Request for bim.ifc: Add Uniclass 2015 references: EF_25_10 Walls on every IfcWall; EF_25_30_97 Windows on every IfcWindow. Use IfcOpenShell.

First a look at what the model holds.

```python
import ifcopenshell

model = ifcopenshell.open("bim.ifc")
print(model.schema)
print("classifications:", [c.Name for c in model.by_type("IfcClassification")])
for ifc_class in ("IfcDoor", "IfcRoof", "IfcStair", "IfcWall", "IfcWindow"):
    print(ifc_class, len(model.by_type(ifc_class)))
```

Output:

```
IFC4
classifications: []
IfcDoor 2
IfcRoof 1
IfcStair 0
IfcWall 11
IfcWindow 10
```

```python
import ifcopenshell
import ifcopenshell.api.classification

model = ifcopenshell.open("bim.ifc")

system = ifcopenshell.api.classification.add_classification(model, classification="Uniclass 2015")

codes = {
    "IfcWall": ("EF_25_10", "Walls"),
    "IfcWindow": ("EF_25_30_97", "Windows"),
}
for ifc_class, (code, name) in codes.items():
    products = model.by_type(ifc_class)
    ifcopenshell.api.classification.add_reference(
        model, products=products, classification=system, identification=code, name=name
    )
    print(code, len(products))

model.write("bim-out.ifc")
```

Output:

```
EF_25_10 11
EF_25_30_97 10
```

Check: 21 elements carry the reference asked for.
